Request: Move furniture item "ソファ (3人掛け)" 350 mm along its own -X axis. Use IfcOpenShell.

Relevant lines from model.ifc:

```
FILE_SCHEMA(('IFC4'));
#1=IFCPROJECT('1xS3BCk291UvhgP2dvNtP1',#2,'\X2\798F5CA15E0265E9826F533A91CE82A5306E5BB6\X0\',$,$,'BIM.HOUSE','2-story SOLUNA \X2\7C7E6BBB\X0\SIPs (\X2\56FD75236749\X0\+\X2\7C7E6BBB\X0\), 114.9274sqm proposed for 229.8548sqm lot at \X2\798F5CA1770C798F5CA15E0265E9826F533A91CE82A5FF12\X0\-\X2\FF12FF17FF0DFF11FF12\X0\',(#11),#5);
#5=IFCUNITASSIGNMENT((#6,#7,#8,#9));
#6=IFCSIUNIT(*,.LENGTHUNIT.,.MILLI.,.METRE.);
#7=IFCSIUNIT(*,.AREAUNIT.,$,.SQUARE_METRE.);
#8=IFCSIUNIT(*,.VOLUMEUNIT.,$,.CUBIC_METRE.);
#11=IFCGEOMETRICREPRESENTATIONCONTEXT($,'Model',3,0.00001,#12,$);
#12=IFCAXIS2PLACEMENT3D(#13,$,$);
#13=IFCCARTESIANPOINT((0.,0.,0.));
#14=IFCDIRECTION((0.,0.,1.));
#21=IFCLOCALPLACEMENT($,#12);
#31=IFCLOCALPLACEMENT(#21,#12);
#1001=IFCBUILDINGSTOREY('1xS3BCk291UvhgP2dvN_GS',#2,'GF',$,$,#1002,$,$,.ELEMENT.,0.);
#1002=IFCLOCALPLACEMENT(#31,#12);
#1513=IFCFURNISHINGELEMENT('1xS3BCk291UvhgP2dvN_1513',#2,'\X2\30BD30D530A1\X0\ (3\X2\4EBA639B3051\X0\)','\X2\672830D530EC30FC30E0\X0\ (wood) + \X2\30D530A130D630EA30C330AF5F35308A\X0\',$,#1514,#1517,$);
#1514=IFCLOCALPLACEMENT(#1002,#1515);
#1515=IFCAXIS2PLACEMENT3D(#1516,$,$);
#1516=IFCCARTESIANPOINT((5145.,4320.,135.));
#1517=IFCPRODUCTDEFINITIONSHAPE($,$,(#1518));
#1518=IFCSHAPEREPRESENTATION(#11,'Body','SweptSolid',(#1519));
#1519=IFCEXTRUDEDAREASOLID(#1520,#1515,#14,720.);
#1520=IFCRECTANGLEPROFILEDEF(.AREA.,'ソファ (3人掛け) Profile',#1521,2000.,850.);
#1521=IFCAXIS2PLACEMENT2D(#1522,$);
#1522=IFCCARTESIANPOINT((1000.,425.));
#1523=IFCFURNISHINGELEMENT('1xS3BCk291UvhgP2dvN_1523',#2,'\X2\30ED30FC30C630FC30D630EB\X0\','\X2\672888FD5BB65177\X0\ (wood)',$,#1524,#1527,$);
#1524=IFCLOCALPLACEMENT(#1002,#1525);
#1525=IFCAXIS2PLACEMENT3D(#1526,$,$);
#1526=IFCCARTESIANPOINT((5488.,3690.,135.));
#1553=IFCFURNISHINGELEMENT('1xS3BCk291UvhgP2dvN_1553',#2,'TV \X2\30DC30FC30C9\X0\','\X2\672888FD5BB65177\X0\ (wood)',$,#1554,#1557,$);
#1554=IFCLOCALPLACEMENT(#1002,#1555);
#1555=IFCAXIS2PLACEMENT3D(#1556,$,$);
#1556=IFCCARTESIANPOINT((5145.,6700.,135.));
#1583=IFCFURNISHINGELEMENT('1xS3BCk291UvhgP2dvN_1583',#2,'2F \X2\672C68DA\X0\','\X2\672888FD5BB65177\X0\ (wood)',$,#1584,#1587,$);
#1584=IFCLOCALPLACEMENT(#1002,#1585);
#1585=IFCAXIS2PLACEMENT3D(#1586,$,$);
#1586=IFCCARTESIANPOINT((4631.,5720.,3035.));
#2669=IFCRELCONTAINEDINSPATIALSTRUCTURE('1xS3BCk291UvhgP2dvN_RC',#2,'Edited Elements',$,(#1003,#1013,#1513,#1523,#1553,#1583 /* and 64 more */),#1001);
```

```python
import ifcopenshell
import ifcopenshell.api.geometry
import ifcopenshell.util.placement
import ifcopenshell.util.unit

model = ifcopenshell.open("model.ifc")
unit_scale = ifcopenshell.util.unit.calculate_unit_scale(model)

item = model.by_guid("1xS3BCk291UvhgP2dvN_1513")
matrix = ifcopenshell.util.placement.get_local_placement(item.ObjectPlacement)
matrix[:3, 3] -= matrix[:3, 0] * 0.35 / unit_scale
ifcopenshell.api.geometry.edit_object_placement(model, product=item, matrix=matrix, is_si=False)

print(ifcopenshell.util.placement.get_local_placement(item.ObjectPlacement).round(3) + 0.0)

model.write("model-out.ifc")
```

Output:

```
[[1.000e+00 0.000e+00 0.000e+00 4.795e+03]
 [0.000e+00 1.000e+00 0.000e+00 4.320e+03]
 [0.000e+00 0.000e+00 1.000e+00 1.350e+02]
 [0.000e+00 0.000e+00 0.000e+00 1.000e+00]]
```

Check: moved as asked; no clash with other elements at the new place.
